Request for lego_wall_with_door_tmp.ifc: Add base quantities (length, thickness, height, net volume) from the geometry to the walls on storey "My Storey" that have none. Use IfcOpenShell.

First a look at what the model holds.

```python
import ifcopenshell
import ifcopenshell.util.element
import ifcopenshell.util.unit

model = ifcopenshell.open("lego_wall_with_door_tmp.ifc")
print(model.schema)
for unit_type in ("LENGTHUNIT", "AREAUNIT", "VOLUMEUNIT"):
    print(unit_type, ifcopenshell.util.unit.calculate_unit_scale(model, unit_type))
storey = next(s for s in model.by_type("IfcBuildingStorey") if s.Name == "My Storey")
walls = [e for e in ifcopenshell.util.element.get_decomposition(storey) if e.is_a("IfcWall")]
for e in sorted(walls, key=lambda e: e.id()):
    print(e.id(), e.is_a(), e.Name, list(ifcopenshell.util.element.get_psets(e, qtos_only=True)), sep=" | ")
```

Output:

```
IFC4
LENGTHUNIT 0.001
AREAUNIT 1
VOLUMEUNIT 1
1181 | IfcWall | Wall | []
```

```python
import ifcopenshell
import ifcopenshell.api.pset
import ifcopenshell.geom
import ifcopenshell.util.element
import ifcopenshell.util.shape
import ifcopenshell.util.unit

model = ifcopenshell.open("lego_wall_with_door_tmp.ifc")
unit_scale = ifcopenshell.util.unit.calculate_unit_scale(model)
volume_scale = ifcopenshell.util.unit.calculate_unit_scale(model, "VOLUMEUNIT")
settings = ifcopenshell.geom.settings()

storey = next(s for s in model.by_type("IfcBuildingStorey") if s.Name == "My Storey")
walls = [e for e in ifcopenshell.util.element.get_decomposition(storey) if e.is_a("IfcWall")]

for e in sorted(walls, key=lambda e: e.id()):
    if ifcopenshell.util.element.get_psets(e, qtos_only=True, should_inherit=False):
        continue
    # Geometry comes back in metres, in the element's own axes.
    shape = ifcopenshell.geom.create_shape(settings, e)
    values = {
        "Length": ifcopenshell.util.shape.get_x(shape.geometry) / unit_scale,
        "Width": ifcopenshell.util.shape.get_y(shape.geometry) / unit_scale,
        "Height": ifcopenshell.util.shape.get_z(shape.geometry) / unit_scale,
        "NetVolume": ifcopenshell.util.shape.get_volume(shape.geometry) / volume_scale,
    }
    qto = ifcopenshell.api.pset.add_qto(model, product=e, name="Qto_WallBaseQuantities")
    ifcopenshell.api.pset.edit_qto(model, qto=qto, properties=values)
    print(e.id(), {k: round(v, 3) for k, v in values.items()})

model.write("lego_wall_with_door_tmp_rev.ifc")
```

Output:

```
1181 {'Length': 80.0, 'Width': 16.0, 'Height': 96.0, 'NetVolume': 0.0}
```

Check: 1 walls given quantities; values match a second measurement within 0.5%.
